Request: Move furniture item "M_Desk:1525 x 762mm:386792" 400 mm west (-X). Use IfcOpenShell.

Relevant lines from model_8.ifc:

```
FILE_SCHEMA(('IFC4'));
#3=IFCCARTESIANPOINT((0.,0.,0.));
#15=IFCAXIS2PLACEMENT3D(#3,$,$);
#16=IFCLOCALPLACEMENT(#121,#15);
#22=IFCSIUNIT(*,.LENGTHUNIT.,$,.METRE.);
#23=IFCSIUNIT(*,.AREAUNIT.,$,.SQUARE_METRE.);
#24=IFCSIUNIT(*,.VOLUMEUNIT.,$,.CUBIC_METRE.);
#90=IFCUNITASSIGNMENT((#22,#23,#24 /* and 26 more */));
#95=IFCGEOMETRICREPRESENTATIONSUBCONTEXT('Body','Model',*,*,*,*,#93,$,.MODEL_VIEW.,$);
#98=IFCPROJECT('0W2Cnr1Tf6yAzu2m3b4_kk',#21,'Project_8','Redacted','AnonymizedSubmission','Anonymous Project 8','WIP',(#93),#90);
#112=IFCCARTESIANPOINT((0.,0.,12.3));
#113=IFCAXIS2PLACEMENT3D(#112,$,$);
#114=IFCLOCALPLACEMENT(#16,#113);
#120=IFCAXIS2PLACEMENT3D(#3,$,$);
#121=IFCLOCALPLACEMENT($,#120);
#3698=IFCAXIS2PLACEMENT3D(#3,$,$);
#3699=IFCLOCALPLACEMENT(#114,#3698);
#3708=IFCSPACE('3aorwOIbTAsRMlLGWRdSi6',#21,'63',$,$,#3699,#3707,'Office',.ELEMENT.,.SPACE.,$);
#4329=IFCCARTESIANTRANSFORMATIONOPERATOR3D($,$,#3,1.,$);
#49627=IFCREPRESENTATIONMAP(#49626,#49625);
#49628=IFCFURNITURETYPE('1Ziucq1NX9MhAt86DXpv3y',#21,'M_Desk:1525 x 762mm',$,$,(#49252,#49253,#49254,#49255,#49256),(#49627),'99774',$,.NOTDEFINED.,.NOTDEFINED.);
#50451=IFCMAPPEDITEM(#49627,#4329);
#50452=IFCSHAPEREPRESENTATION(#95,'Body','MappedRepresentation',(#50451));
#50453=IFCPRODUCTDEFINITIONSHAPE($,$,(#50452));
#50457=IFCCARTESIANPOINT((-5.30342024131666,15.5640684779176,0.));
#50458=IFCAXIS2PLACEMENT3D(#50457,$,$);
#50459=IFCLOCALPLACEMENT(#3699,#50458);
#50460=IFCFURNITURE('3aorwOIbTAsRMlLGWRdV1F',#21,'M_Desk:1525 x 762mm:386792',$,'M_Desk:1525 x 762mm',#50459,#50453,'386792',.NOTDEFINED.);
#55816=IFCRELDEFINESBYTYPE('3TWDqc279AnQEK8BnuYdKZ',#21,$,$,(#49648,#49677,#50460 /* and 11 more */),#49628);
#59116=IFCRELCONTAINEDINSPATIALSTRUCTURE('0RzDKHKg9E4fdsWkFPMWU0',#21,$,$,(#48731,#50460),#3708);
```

```python
import ifcopenshell
import ifcopenshell.api.geometry
import ifcopenshell.util.placement

model = ifcopenshell.open("model_8.ifc")

item = model.by_guid("3aorwOIbTAsRMlLGWRdV1F")
matrix = ifcopenshell.util.placement.get_local_placement(item.ObjectPlacement)
matrix[0, 3] -= 0.4
ifcopenshell.api.geometry.edit_object_placement(model, product=item, matrix=matrix, is_si=False)

print(ifcopenshell.util.placement.get_local_placement(item.ObjectPlacement).round(3) + 0.0)

model.write("model_8_v2.ifc")
```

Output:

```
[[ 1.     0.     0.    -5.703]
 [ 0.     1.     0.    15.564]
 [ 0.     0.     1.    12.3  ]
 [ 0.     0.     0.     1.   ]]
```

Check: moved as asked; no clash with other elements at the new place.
